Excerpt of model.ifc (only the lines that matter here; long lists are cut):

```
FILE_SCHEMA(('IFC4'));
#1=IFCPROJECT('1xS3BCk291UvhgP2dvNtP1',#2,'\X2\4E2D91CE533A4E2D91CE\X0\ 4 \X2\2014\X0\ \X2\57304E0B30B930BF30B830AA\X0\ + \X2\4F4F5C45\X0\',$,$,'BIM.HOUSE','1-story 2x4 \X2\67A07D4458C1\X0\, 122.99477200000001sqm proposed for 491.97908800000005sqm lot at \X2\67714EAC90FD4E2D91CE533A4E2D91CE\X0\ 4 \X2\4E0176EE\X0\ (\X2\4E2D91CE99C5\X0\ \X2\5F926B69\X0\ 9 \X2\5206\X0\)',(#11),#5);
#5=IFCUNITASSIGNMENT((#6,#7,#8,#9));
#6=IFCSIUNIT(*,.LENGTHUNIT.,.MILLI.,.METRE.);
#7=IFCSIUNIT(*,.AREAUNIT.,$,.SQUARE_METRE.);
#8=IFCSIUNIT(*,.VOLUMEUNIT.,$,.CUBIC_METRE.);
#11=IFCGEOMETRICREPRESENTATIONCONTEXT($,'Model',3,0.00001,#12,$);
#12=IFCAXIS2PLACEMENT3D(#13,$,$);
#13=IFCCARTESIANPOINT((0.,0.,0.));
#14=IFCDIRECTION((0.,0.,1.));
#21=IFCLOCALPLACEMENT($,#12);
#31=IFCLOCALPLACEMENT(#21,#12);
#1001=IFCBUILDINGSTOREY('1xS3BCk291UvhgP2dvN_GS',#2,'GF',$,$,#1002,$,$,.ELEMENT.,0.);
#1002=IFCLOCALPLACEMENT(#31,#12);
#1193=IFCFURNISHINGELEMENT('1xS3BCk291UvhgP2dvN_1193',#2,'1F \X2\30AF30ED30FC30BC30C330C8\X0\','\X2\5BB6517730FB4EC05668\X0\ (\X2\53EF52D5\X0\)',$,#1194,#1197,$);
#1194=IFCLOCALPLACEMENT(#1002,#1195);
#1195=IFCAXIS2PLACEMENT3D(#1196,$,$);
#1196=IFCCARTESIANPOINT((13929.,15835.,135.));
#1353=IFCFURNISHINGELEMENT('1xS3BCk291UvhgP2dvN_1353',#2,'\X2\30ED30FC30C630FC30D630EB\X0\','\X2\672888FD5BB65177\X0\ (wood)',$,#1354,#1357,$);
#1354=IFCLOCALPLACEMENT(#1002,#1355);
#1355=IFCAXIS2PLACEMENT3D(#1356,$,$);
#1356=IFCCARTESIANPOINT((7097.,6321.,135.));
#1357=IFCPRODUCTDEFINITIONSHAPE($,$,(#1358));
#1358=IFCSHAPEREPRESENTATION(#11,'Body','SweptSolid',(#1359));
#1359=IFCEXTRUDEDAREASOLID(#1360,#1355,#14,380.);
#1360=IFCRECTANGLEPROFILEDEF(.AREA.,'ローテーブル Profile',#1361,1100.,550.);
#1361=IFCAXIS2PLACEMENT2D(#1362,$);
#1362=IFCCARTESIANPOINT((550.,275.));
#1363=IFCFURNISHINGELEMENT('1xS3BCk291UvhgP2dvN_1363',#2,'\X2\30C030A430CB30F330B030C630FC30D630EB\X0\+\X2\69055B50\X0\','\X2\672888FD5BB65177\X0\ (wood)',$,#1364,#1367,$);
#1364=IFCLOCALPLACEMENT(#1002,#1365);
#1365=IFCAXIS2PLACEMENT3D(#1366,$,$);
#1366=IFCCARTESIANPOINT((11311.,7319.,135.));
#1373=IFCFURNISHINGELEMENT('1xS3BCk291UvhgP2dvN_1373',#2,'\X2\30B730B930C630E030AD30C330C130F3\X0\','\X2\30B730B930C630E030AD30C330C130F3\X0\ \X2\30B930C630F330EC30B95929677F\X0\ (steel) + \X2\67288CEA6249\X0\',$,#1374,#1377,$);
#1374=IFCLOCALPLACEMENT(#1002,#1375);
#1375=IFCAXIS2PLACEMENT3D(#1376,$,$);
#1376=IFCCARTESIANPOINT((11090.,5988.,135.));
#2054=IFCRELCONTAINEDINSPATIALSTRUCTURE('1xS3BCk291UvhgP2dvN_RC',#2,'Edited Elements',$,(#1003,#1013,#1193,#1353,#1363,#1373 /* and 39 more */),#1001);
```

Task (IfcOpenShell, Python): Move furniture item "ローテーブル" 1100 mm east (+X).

```python
import ifcopenshell
import ifcopenshell.api.geometry
import ifcopenshell.util.placement
import ifcopenshell.util.unit

model = ifcopenshell.open("model.ifc")
unit_scale = ifcopenshell.util.unit.calculate_unit_scale(model)

item = model.by_id(1353)
matrix = ifcopenshell.util.placement.get_local_placement(item.ObjectPlacement)
matrix[0, 3] += 1.1 / unit_scale
ifcopenshell.api.geometry.edit_object_placement(model, product=item, matrix=matrix, is_si=False)

print(ifcopenshell.util.placement.get_local_placement(item.ObjectPlacement).round(3) + 0.0)

model.write("model_v2.ifc")
```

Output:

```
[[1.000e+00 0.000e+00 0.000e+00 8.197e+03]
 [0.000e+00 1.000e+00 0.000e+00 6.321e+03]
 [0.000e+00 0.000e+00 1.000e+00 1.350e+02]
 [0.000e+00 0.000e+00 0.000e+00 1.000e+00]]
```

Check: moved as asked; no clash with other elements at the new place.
